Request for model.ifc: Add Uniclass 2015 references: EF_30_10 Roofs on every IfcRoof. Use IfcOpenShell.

First a look at what the model holds.

```python
import ifcopenshell

model = ifcopenshell.open("model.ifc")
print(model.schema)
print("classifications:", [c.Name for c in model.by_type("IfcClassification")])
for ifc_class in ("IfcDoor", "IfcRoof", "IfcStair", "IfcWall", "IfcWindow"):
    print(ifc_class, len(model.by_type(ifc_class)))
```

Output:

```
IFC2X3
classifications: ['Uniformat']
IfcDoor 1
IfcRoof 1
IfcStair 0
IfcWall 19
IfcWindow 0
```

```python
import ifcopenshell
import ifcopenshell.api.classification

model = ifcopenshell.open("model.ifc")

# IFC2X3 requires Source and Edition and has no link from the project to the system.
system = model.create_entity("IfcClassification", Source="NBS", Edition="2015", Name="Uniclass 2015")

codes = {
    "IfcRoof": ("EF_30_10", "Roofs"),
}
for ifc_class, (code, name) in codes.items():
    products = model.by_type(ifc_class)
    ifcopenshell.api.classification.add_reference(
        model, products=products, classification=system, identification=code, name=name
    )
    print(code, len(products))

model.write("model_updated.ifc")
```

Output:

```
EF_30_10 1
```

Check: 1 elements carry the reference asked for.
